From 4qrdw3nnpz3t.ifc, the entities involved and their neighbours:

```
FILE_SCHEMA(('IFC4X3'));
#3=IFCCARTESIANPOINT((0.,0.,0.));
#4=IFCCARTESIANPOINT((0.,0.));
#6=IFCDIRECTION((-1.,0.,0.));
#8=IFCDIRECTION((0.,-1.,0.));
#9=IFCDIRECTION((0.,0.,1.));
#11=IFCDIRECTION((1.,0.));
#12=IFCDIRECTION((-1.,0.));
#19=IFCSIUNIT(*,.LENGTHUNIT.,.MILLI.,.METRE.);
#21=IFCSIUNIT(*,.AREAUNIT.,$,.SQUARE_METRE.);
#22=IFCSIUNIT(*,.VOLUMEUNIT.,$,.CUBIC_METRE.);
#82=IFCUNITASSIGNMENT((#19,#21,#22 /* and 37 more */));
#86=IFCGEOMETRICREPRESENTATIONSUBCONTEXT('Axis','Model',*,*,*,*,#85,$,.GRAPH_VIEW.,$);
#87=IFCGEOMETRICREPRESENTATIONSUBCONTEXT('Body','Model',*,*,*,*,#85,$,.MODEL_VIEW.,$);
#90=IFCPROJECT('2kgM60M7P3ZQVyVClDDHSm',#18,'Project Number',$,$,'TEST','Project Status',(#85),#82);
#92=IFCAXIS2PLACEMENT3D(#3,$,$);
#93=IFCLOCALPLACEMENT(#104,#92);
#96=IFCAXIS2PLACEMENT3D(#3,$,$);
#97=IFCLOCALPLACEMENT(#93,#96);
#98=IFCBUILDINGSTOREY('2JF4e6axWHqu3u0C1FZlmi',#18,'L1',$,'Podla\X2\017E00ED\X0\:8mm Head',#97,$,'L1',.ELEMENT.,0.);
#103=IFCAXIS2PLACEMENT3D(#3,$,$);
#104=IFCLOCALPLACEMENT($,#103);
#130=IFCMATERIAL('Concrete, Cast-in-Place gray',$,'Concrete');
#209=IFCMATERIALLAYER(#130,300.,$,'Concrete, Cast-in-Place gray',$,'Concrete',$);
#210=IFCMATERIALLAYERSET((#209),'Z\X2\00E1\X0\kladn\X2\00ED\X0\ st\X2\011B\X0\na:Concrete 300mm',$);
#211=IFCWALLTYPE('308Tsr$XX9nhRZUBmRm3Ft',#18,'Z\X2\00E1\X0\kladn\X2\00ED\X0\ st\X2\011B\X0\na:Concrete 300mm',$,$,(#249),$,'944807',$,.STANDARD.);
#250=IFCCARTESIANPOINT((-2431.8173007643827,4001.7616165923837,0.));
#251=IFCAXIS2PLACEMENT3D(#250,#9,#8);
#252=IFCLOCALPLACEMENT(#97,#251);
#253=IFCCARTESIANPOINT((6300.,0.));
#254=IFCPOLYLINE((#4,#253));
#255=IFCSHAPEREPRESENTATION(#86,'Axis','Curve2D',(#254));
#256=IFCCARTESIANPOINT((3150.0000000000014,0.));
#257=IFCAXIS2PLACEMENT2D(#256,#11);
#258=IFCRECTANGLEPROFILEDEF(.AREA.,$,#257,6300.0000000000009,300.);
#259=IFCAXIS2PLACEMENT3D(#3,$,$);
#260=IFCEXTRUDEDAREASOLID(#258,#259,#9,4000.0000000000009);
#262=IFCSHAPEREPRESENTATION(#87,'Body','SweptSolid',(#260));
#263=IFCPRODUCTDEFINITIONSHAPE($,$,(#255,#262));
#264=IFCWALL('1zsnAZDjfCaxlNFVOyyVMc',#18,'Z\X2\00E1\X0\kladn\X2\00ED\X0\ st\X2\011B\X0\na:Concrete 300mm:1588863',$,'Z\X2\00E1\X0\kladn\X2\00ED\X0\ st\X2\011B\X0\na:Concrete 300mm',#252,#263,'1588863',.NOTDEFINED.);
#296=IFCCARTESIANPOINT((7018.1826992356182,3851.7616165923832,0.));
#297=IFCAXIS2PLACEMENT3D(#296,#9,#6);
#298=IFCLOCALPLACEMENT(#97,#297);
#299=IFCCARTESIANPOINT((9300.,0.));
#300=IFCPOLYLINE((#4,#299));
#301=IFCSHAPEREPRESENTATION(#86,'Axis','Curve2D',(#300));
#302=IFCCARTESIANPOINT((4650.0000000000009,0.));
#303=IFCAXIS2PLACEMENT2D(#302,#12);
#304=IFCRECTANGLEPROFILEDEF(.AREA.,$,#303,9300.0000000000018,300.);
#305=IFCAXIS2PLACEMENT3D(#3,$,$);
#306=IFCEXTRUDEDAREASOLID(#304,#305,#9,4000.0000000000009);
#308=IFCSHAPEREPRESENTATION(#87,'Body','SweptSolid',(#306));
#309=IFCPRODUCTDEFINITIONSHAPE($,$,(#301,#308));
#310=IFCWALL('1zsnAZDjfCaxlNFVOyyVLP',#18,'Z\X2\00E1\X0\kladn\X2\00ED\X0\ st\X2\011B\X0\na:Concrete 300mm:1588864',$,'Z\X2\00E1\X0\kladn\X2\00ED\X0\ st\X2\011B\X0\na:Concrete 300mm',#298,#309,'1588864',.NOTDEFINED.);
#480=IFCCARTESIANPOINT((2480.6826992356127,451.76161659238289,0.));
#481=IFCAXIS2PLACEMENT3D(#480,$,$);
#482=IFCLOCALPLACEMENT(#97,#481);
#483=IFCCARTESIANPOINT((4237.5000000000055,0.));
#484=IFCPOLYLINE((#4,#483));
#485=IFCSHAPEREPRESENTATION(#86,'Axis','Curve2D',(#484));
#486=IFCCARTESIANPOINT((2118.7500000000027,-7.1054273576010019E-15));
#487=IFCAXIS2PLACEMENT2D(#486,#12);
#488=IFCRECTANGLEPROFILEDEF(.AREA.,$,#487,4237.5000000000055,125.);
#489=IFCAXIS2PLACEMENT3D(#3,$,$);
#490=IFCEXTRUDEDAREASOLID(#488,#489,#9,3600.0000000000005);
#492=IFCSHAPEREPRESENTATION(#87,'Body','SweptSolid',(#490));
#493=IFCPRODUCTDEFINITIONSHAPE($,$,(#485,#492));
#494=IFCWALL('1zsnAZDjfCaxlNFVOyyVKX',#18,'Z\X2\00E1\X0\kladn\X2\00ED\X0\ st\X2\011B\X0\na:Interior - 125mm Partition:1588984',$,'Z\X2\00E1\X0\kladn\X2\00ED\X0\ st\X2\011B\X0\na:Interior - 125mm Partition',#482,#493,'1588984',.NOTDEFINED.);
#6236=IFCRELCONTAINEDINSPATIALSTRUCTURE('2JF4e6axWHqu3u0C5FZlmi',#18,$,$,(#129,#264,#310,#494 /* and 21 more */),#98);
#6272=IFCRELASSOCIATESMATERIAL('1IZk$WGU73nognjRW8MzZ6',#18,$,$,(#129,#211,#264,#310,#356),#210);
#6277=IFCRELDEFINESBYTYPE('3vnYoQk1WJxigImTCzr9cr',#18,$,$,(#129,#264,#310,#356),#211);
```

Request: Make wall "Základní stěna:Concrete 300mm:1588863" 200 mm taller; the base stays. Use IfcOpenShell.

```python
import ifcopenshell
import ifcopenshell.geom
import ifcopenshell.util.representation
import ifcopenshell.util.shape
import ifcopenshell.util.unit

model = ifcopenshell.open("4qrdw3nnpz3t.ifc")
unit_scale = ifcopenshell.util.unit.calculate_unit_scale(model)
settings = ifcopenshell.geom.settings()


def volume(element):
    """Net volume in cubic metres, openings subtracted."""
    shape = ifcopenshell.geom.create_shape(settings, element)
    return ifcopenshell.util.shape.get_volume(shape.geometry)


wall = model.by_guid("1zsnAZDjfCaxlNFVOyyVMc")
before = volume(wall)

body = ifcopenshell.util.representation.get_representation(wall, "Model", "Body")
solid = body.Items[0]
old_height = solid.Depth
solid.Depth += 0.2 / unit_scale
after = volume(wall)

print(f"height {old_height:g} -> {solid.Depth:g}, volume {before:.3f} -> {after:.3f} m3")

model.write("4qrdw3nnpz3t-out.ifc")
```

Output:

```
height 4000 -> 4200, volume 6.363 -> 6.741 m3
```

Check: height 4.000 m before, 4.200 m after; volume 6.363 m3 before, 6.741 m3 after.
